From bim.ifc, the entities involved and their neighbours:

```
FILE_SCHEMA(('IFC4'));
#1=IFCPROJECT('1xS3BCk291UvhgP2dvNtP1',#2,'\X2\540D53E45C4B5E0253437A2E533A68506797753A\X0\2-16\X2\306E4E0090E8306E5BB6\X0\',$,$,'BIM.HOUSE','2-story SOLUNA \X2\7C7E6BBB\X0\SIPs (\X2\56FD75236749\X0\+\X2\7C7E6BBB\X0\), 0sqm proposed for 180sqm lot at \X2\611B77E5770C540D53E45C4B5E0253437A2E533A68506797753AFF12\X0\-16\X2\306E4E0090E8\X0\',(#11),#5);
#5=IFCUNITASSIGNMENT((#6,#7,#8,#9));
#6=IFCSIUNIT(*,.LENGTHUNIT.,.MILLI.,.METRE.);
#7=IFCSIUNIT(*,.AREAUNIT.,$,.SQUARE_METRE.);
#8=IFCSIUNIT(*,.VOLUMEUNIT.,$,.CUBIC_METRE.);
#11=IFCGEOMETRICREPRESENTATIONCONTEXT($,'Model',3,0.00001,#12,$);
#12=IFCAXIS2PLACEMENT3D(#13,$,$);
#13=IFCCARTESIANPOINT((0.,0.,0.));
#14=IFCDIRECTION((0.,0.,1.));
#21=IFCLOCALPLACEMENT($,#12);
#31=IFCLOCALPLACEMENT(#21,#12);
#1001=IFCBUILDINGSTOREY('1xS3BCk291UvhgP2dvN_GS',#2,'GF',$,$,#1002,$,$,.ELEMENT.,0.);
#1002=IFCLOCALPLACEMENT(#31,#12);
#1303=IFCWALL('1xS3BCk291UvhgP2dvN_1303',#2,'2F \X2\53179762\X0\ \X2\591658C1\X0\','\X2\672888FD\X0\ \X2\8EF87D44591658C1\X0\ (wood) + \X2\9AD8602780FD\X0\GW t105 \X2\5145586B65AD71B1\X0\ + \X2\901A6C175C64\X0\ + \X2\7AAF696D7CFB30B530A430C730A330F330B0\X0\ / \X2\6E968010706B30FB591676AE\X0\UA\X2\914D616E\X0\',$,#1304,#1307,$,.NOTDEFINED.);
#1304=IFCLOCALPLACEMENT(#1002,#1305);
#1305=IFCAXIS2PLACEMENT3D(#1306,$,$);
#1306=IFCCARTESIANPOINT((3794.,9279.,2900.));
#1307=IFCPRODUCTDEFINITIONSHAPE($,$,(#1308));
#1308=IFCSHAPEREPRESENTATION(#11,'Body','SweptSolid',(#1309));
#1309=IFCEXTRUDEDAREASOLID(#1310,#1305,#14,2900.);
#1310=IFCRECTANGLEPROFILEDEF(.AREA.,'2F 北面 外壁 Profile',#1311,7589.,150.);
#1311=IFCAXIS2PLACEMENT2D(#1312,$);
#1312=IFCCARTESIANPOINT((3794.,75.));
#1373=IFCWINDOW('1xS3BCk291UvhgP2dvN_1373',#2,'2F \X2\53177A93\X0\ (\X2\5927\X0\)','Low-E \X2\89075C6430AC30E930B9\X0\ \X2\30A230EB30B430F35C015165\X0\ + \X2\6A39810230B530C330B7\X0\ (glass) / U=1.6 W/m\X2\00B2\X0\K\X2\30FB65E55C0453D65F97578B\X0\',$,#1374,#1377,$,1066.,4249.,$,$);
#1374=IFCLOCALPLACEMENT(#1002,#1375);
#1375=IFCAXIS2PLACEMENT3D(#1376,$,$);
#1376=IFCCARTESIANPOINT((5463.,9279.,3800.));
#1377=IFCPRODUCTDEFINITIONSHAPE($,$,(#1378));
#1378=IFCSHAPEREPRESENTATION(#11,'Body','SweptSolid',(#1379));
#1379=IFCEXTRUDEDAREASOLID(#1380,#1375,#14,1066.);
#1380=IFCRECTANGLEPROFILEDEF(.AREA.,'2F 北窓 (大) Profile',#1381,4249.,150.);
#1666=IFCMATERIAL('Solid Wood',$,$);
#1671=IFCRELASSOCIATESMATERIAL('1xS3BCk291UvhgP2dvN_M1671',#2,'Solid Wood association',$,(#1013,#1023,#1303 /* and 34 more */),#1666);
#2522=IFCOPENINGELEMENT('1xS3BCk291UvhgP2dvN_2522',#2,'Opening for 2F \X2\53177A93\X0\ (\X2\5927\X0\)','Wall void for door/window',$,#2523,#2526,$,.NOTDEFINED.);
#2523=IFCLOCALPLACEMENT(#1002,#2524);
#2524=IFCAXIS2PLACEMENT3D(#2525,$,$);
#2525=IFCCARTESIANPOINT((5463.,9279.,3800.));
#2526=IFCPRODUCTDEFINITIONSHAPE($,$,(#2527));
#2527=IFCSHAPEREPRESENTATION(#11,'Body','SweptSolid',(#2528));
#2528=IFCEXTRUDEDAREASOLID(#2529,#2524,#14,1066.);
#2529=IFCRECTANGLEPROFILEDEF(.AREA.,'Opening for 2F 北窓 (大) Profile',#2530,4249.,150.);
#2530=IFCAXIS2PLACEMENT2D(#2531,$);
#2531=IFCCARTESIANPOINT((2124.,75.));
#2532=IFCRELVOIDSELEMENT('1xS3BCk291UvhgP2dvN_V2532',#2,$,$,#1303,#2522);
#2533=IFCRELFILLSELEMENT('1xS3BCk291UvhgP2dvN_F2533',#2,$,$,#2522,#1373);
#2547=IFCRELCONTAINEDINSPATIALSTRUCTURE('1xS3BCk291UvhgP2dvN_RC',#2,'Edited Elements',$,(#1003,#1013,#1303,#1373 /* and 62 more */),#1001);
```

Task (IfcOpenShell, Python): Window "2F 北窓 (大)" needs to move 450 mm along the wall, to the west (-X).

```python
import ifcopenshell
import ifcopenshell.api.geometry
import ifcopenshell.util.placement
import ifcopenshell.util.unit

model = ifcopenshell.open("bim.ifc")
unit_scale = ifcopenshell.util.unit.calculate_unit_scale(model)

window = model.by_guid("1xS3BCk291UvhgP2dvN_1373")
opening = window.FillsVoids[0].RelatingOpeningElement
wall = opening.VoidsElements[0].RelatingBuildingElement

wall_matrix = ifcopenshell.util.placement.get_local_placement(wall.ObjectPlacement)
shift = wall_matrix[:3, 0] * -0.45 / unit_scale
before = ifcopenshell.util.placement.get_local_placement(window.ObjectPlacement)[:3, 3].copy()

# The window is not placed relative to its opening, so move both.
for product in (opening, window):
    matrix = ifcopenshell.util.placement.get_local_placement(product.ObjectPlacement)
    matrix[:3, 3] += shift
    ifcopenshell.api.geometry.edit_object_placement(model, product=product, matrix=matrix, is_si=False)

after = ifcopenshell.util.placement.get_local_placement(window.ObjectPlacement)[:3, 3]
print("window moved by", (after - before).round(3) + 0.0)

model.write("bim_updated.ifc")
```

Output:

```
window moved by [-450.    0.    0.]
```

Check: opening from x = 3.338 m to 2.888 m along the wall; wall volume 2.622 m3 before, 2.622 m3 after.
